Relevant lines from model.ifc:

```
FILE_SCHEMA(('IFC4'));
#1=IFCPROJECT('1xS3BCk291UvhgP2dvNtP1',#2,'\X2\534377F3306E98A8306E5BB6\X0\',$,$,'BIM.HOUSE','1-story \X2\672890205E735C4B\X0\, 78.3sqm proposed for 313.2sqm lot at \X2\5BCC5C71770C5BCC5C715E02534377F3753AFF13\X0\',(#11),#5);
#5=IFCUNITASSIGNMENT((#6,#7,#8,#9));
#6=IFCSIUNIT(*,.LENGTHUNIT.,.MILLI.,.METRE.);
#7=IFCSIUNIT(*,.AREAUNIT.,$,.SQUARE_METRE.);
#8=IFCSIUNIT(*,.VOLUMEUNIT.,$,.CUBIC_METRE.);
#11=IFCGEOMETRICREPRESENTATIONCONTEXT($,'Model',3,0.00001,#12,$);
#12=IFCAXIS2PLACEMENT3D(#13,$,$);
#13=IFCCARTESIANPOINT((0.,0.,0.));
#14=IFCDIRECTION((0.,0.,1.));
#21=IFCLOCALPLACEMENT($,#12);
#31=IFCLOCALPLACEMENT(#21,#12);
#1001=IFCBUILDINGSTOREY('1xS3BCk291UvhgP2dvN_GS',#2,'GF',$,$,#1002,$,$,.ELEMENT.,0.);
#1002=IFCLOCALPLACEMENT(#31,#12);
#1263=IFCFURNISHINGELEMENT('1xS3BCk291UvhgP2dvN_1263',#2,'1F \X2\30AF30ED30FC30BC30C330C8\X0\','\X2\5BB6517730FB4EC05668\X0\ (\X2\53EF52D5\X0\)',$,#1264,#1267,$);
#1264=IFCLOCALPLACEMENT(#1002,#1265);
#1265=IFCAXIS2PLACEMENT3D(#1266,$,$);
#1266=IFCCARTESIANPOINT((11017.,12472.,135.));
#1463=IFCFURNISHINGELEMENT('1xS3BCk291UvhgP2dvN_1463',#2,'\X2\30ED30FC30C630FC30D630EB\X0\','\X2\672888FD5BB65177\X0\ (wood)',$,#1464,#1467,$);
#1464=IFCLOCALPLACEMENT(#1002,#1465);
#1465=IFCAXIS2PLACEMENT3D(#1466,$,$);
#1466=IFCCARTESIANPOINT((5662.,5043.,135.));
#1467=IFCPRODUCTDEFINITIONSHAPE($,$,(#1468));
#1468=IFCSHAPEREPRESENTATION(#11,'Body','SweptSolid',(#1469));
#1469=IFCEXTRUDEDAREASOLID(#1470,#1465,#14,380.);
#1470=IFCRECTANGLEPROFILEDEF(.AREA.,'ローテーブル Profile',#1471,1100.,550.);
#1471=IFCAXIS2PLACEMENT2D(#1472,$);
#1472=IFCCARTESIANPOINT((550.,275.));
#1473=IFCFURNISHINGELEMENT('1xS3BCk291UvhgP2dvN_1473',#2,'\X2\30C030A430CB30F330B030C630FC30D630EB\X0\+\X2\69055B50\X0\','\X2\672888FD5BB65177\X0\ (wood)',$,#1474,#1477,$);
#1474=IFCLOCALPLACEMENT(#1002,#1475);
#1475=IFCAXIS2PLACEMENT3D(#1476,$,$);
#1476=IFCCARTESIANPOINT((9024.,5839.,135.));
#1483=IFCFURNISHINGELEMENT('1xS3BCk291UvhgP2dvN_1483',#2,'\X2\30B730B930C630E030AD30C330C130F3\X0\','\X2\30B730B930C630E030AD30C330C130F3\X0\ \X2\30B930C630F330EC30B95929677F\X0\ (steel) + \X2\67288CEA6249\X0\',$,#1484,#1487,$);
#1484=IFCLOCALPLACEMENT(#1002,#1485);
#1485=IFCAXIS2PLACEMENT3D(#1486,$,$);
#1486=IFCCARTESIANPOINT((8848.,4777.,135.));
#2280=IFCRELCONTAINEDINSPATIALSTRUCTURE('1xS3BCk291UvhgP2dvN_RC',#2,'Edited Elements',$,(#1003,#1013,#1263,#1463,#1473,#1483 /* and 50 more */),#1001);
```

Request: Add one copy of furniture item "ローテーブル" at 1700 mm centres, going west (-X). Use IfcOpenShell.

```python
import numpy as np
import ifcopenshell
import ifcopenshell.api.geometry
import ifcopenshell.api.root
import ifcopenshell.util.element
import ifcopenshell.util.placement

model = ifcopenshell.open("model.ifc")


def reuse_history(source, copy):
    """copy_class also copies each property set's owner history, people and application; keep the originals."""
    for rel in copy.IsDefinedBy:
        if rel.is_a("IfcRelDefinesByProperties") and (history := rel.RelatingPropertyDefinition.OwnerHistory):
            rel.RelatingPropertyDefinition.OwnerHistory = source.OwnerHistory
            ifcopenshell.util.element.remove_deep2(model, history)


source = model.by_id(1463)
base = ifcopenshell.util.placement.get_local_placement(source.ObjectPlacement)
step = np.array([-1.0, 0.0, 0.0]) * 1700.0

for i in range(1, 2):
    copy = ifcopenshell.api.root.copy_class(model, product=source)
    copy.Representation = ifcopenshell.util.element.copy_deep(
        model, source.Representation, exclude=["IfcGeometricRepresentationContext", "IfcRepresentationMap"]
    )
    reuse_history(source, copy)
    matrix = base.copy()
    matrix[:3, 3] += i * step
    print("added at", matrix[:3, 3].round(3) + 0.0)
    ifcopenshell.api.geometry.edit_object_placement(model, product=copy, matrix=matrix, is_si=False)

model.write("model_updated.ifc")
```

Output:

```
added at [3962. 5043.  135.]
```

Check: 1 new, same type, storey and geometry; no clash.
